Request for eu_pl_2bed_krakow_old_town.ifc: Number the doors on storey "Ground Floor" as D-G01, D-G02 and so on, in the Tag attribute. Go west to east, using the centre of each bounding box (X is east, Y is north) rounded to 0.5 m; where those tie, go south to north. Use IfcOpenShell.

First a look at what the model holds.

```python
import ifcopenshell
import ifcopenshell.util.element
import ifcopenshell.util.placement

model = ifcopenshell.open("eu_pl_2bed_krakow_old_town.ifc")
print(model.schema)
storey = next(s for s in model.by_type("IfcBuildingStorey") if s.Name == "Ground Floor")
doors = [e for e in ifcopenshell.util.element.get_decomposition(storey) if e.is_a("IfcDoor")]
for e in sorted(doors, key=lambda e: e.id()):
    origin = ifcopenshell.util.placement.get_local_placement(e.ObjectPlacement)[:3, 3]
    print(e.id(), e.Tag, e.Name, origin.round(2) + 0.0, sep=" | ")
```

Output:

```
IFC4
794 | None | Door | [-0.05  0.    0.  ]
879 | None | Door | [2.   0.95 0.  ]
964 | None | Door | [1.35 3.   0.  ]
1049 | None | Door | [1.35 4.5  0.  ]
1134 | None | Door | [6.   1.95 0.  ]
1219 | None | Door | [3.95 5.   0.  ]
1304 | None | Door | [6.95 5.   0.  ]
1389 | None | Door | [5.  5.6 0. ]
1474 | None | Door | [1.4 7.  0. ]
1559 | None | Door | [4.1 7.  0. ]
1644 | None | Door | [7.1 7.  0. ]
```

```python
import ifcopenshell
import ifcopenshell.geom
import ifcopenshell.util.element
import ifcopenshell.util.shape

model = ifcopenshell.open("eu_pl_2bed_krakow_old_town.ifc")
settings = ifcopenshell.geom.settings()
settings.set("use-world-coords", True)


def centre(element):
    shape = ifcopenshell.geom.create_shape(settings, element)
    return ifcopenshell.util.shape.get_bbox_centroid(shape.geometry)


storey = next(s for s in model.by_type("IfcBuildingStorey") if s.Name == "Ground Floor")
doors = [e for e in ifcopenshell.util.element.get_decomposition(storey) if e.is_a("IfcDoor")]

# Insertion points can sit at a corner or the storey origin, so sort by the geometry (in metres).
centres = {e: centre(e) for e in doors}
doors.sort(key=lambda e: (round(centres[e][0] / 0.5), centres[e][1]))

for i, e in enumerate(doors, start=1):
    number = f"D-G{i:02d}"
    e.Tag = number
    print(e.id(), number)

model.write("eu_pl_2bed_krakow_old_town_edited.ifc")
```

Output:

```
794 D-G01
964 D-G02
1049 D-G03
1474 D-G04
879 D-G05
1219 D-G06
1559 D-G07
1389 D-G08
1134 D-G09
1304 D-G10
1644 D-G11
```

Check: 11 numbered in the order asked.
